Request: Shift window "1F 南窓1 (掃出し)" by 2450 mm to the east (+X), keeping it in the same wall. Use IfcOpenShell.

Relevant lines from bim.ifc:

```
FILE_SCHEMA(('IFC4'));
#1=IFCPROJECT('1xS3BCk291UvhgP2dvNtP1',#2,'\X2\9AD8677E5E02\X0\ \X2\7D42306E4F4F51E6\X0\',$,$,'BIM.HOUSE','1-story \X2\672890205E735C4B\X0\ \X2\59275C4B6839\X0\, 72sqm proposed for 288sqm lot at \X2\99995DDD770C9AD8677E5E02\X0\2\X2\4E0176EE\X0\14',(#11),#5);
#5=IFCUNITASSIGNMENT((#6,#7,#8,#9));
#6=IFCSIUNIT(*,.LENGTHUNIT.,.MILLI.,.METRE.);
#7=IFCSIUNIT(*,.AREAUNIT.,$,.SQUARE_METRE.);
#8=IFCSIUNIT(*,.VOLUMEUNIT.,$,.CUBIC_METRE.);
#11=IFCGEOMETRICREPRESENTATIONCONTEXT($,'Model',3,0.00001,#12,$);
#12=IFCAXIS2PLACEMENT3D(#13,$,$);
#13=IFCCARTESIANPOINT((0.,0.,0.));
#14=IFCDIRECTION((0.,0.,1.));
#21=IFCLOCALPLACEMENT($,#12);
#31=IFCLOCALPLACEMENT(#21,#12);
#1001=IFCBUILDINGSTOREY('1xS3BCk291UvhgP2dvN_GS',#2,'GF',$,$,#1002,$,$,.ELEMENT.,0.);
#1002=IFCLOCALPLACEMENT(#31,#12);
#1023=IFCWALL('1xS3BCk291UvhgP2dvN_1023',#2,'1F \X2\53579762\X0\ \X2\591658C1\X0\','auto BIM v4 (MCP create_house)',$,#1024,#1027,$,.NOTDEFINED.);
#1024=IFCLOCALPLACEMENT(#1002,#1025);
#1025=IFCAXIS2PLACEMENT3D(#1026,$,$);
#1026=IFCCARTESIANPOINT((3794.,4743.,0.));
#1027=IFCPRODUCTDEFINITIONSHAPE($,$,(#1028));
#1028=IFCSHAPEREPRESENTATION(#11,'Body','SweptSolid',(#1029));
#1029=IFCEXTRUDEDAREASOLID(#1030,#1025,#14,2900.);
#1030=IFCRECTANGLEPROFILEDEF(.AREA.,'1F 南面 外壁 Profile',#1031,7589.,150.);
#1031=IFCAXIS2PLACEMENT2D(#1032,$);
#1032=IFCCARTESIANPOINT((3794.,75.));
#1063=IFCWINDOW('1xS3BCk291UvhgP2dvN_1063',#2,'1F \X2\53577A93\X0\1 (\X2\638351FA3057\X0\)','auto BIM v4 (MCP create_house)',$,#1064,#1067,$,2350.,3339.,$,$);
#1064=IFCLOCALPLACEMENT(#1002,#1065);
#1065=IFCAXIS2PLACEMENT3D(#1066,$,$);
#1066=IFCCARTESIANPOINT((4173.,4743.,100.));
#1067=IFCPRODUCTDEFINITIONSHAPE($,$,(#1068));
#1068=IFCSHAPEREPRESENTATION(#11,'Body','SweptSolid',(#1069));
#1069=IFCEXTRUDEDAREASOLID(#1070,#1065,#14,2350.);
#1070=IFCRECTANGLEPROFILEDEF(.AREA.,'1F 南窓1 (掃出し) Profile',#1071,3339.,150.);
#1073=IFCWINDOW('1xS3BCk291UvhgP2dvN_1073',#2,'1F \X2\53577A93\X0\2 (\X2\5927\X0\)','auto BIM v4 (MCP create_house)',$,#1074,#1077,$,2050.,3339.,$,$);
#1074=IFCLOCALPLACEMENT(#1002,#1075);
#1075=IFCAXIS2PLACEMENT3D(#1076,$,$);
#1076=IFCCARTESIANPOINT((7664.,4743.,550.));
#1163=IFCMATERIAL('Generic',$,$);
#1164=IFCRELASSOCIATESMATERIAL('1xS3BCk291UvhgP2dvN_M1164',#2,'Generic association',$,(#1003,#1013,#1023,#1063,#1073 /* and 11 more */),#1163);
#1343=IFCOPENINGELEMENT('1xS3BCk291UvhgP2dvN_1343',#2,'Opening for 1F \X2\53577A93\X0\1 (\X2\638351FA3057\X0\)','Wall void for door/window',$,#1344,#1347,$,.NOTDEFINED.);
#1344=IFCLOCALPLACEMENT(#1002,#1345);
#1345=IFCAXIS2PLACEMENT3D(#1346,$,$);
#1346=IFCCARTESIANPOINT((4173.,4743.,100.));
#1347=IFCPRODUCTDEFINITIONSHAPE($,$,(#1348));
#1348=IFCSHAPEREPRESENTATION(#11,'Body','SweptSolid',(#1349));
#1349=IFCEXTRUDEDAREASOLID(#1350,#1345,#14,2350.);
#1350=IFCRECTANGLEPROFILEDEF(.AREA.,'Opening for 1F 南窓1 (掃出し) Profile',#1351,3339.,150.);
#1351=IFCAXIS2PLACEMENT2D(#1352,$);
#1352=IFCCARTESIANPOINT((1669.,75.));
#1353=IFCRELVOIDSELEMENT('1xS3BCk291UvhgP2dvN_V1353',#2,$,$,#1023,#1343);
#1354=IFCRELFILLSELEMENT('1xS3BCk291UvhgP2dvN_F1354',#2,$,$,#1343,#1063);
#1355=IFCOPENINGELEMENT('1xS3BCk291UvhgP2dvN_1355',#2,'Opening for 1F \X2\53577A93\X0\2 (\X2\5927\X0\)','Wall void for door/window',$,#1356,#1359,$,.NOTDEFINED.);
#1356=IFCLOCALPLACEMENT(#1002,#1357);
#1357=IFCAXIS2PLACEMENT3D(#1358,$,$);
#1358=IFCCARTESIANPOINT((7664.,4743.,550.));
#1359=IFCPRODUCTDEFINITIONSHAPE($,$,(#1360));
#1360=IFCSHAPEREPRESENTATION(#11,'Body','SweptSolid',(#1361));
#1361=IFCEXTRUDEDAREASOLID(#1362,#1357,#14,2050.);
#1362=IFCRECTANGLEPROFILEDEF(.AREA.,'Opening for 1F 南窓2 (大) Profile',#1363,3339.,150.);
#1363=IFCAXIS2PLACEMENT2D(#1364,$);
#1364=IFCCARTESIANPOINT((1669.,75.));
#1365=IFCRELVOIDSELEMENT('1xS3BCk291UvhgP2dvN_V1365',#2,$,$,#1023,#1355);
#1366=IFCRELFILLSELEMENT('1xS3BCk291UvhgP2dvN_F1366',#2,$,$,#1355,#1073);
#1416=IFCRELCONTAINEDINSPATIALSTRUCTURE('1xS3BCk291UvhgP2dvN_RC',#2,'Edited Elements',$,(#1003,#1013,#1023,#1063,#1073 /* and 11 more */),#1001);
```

```python
import ifcopenshell
import ifcopenshell.api.geometry
import ifcopenshell.util.placement
import ifcopenshell.util.unit

model = ifcopenshell.open("bim.ifc")
unit_scale = ifcopenshell.util.unit.calculate_unit_scale(model)

window = model.by_guid("1xS3BCk291UvhgP2dvN_1063")
opening = window.FillsVoids[0].RelatingOpeningElement
wall = opening.VoidsElements[0].RelatingBuildingElement

wall_matrix = ifcopenshell.util.placement.get_local_placement(wall.ObjectPlacement)
shift = wall_matrix[:3, 0] * 2.45 / unit_scale
before = ifcopenshell.util.placement.get_local_placement(window.ObjectPlacement)[:3, 3].copy()

# The window is not placed relative to its opening, so move both.
for product in (opening, window):
    matrix = ifcopenshell.util.placement.get_local_placement(product.ObjectPlacement)
    matrix[:3, 3] += shift
    ifcopenshell.api.geometry.edit_object_placement(model, product=product, matrix=matrix, is_si=False)

after = ifcopenshell.util.placement.get_local_placement(window.ObjectPlacement)[:3, 3]
print("window moved by", (after - before).round(3) + 0.0)

model.write("bim-out.ifc")
```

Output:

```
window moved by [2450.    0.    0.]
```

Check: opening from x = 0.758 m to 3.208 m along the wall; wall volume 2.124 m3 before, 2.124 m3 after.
